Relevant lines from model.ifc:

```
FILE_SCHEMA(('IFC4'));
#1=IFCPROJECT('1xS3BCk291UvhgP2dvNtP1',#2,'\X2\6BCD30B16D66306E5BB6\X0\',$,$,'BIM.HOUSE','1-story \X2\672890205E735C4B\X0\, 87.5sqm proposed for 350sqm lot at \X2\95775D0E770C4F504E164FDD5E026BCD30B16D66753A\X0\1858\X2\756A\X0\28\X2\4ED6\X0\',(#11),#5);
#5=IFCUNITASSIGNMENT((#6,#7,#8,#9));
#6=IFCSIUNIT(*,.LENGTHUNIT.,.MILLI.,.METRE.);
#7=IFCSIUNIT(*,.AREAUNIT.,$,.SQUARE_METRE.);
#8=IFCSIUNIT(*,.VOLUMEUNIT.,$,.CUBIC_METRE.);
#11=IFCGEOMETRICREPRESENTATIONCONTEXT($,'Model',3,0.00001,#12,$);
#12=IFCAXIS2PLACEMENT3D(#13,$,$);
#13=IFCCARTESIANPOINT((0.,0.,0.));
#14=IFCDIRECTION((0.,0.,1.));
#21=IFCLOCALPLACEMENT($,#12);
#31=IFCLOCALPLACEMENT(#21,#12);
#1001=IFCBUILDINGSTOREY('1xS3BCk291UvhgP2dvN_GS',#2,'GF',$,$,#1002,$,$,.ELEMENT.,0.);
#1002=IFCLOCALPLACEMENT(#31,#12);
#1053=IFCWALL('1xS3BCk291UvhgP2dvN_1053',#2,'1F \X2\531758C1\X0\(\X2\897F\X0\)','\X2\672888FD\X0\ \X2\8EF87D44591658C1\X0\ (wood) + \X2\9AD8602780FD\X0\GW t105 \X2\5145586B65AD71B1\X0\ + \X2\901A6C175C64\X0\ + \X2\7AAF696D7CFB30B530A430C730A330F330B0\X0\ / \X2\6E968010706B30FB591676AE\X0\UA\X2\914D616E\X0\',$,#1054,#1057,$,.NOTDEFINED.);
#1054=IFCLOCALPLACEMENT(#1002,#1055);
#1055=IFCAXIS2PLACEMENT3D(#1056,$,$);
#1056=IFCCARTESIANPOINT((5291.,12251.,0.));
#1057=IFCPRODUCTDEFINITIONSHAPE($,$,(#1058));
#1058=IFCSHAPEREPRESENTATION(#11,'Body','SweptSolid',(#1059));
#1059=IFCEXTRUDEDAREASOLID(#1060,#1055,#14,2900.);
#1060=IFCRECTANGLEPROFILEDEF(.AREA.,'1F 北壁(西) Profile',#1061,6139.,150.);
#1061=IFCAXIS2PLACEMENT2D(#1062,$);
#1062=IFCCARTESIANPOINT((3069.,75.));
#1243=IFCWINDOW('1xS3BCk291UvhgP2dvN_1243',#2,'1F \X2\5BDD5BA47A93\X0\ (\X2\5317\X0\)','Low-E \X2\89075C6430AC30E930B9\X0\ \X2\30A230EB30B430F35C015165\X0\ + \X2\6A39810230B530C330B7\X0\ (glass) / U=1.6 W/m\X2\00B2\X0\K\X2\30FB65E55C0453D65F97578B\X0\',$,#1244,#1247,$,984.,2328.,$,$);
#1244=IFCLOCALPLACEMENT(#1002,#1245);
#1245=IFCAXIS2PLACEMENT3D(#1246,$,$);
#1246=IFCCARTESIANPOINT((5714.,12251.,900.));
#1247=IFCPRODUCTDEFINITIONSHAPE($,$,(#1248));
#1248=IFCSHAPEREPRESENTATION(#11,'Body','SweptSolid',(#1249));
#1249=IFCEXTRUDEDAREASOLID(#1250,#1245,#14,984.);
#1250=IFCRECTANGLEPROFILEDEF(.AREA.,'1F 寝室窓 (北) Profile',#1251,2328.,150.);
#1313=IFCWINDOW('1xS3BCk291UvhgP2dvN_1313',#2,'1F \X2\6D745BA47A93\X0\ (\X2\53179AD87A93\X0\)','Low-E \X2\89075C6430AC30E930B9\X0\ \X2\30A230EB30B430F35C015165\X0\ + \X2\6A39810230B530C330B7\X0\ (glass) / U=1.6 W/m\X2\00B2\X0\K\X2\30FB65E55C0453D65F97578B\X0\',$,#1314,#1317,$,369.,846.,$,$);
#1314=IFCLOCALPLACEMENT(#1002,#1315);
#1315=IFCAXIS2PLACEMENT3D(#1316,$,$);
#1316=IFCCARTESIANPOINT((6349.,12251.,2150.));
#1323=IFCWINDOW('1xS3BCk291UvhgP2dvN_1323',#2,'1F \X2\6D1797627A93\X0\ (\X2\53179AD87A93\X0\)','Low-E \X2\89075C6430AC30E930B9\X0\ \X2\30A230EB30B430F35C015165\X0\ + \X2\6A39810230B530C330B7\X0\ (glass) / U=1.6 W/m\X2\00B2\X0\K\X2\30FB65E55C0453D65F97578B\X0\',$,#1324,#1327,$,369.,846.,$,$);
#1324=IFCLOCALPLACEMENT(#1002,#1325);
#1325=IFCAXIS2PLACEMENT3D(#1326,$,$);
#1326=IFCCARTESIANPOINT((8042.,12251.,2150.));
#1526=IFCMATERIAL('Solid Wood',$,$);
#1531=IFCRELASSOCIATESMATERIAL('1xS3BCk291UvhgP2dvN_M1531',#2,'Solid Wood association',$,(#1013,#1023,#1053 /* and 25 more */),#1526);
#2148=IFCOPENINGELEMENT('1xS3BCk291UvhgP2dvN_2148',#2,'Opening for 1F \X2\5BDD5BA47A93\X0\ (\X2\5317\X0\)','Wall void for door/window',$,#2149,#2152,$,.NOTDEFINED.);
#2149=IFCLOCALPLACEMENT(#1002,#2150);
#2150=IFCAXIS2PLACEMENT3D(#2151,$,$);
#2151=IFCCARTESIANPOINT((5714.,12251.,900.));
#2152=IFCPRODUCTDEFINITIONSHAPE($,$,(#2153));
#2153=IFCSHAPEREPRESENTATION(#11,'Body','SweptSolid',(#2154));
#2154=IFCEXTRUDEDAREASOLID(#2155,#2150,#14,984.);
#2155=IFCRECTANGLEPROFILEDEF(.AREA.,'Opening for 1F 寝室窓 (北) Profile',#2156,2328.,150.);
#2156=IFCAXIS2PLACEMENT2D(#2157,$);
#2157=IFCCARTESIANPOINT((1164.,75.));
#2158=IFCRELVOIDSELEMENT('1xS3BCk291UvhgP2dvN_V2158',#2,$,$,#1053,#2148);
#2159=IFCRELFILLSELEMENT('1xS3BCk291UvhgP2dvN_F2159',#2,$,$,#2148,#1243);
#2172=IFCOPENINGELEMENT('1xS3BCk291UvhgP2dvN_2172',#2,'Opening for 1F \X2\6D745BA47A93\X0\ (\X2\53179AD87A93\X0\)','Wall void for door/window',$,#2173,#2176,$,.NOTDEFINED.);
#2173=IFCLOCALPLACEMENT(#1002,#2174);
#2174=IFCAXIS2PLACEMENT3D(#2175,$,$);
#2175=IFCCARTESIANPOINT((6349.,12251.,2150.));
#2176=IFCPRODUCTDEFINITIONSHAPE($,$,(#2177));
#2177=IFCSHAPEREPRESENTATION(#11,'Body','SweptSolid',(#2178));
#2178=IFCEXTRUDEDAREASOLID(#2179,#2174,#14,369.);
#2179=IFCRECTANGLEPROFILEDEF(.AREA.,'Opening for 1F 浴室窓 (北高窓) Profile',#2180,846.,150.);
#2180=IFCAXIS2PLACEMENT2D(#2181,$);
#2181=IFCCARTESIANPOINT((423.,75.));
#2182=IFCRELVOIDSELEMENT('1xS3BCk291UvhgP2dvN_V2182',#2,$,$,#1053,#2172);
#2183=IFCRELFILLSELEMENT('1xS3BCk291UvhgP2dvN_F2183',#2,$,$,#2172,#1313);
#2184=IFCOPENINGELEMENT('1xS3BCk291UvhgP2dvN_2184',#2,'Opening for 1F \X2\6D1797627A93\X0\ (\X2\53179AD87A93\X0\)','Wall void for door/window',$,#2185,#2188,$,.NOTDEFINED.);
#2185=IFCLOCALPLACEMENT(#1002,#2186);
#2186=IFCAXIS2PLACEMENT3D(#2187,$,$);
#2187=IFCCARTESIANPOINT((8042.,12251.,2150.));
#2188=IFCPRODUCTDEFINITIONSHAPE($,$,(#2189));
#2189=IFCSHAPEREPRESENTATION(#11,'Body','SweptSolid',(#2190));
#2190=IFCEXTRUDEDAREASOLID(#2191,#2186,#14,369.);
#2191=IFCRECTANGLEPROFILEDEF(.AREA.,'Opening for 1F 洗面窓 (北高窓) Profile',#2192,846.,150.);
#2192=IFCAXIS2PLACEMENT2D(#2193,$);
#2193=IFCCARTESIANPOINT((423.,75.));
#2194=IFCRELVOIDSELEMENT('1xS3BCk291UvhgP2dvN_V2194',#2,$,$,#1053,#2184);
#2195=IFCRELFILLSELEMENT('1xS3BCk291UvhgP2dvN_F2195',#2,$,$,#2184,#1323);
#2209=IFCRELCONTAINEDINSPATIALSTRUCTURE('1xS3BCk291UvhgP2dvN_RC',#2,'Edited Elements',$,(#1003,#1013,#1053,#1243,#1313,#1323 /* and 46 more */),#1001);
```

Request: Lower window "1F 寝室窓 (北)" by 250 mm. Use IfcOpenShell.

```python
import numpy as np
import ifcopenshell
import ifcopenshell.api.geometry
import ifcopenshell.util.placement
import ifcopenshell.util.unit

model = ifcopenshell.open("model.ifc")
unit_scale = ifcopenshell.util.unit.calculate_unit_scale(model)

window = model.by_id(1243)
opening = window.FillsVoids[0].RelatingOpeningElement
dz = -0.25 / unit_scale

shift = np.array([0.0, 0.0, dz])
# The window is not placed relative to its opening, so move both.
for product in (opening, window):
    matrix = ifcopenshell.util.placement.get_local_placement(product.ObjectPlacement)
    matrix[:3, 3] += shift
    ifcopenshell.api.geometry.edit_object_placement(model, product=product, matrix=matrix, is_si=False)

print(f"moved by {dz * unit_scale:+.3f} m")

model.write("model_rev.ifc")
```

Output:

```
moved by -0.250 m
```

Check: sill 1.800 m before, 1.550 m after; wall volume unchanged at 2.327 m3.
